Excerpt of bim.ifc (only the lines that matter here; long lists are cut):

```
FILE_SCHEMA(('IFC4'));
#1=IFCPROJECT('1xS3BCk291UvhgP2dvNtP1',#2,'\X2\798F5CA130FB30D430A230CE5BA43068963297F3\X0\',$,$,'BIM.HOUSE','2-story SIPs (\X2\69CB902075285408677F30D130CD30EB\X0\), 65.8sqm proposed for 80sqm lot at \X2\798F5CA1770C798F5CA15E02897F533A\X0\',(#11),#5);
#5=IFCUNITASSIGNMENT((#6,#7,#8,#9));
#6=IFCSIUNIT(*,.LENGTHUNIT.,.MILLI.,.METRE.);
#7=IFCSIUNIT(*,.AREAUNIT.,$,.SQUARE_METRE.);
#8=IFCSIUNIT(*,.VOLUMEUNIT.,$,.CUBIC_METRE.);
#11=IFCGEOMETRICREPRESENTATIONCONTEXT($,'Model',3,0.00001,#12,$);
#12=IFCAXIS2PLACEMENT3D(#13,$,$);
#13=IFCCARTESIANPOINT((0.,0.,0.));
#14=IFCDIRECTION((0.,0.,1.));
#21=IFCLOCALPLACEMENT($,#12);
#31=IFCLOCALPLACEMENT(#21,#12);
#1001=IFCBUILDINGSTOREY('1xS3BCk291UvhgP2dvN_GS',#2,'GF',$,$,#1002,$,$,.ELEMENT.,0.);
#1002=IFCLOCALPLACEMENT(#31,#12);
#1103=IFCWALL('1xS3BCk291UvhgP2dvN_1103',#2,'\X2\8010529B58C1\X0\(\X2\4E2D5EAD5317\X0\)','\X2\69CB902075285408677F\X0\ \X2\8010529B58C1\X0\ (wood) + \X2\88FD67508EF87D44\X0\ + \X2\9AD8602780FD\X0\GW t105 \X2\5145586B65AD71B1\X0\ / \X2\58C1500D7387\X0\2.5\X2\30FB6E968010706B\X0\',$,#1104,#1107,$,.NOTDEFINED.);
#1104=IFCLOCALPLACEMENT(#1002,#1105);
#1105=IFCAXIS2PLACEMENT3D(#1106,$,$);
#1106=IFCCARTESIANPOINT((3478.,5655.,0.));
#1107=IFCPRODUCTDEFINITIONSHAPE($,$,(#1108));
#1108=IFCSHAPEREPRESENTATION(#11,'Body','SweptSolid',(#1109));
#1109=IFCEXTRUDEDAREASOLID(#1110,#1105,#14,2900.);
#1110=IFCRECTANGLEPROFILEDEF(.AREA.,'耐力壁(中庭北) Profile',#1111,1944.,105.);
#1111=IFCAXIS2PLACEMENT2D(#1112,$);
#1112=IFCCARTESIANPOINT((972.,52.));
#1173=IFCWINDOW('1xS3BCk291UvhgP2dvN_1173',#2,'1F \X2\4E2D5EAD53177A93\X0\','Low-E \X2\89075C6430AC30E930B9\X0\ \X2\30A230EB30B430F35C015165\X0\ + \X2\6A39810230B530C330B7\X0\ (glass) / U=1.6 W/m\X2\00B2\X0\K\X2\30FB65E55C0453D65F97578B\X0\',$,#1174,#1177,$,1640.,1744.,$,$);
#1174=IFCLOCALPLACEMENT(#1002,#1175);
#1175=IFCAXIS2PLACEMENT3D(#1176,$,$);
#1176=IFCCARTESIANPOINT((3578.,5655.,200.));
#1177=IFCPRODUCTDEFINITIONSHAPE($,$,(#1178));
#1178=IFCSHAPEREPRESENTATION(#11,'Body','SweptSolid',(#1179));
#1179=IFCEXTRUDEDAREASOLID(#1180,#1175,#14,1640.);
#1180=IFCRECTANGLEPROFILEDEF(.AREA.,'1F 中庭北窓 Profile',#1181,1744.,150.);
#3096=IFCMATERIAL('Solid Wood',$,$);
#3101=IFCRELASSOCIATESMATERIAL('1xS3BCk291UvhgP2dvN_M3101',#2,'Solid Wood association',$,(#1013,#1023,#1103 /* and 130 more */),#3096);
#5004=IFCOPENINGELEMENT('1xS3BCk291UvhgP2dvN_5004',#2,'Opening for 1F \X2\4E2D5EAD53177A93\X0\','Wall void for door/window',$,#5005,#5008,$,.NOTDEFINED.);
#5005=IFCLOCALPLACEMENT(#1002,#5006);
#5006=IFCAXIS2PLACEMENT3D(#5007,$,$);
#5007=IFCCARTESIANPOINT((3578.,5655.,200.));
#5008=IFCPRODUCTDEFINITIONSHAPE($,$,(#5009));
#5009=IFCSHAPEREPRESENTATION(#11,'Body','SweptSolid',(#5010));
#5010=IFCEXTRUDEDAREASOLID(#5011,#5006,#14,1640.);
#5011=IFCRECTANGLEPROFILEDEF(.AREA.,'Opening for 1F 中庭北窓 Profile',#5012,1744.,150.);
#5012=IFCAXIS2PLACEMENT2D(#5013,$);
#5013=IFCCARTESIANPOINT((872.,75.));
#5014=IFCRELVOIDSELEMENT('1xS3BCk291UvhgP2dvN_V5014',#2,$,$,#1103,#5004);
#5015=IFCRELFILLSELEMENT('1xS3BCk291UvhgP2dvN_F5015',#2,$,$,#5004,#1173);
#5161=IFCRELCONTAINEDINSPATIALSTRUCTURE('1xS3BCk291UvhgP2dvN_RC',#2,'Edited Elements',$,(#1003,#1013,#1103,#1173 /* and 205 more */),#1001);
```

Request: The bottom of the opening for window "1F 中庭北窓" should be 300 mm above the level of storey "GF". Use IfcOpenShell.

```python
import numpy as np
import ifcopenshell
import ifcopenshell.api.geometry
import ifcopenshell.geom
import ifcopenshell.util.element
import ifcopenshell.util.placement
import ifcopenshell.util.shape
import ifcopenshell.util.unit

model = ifcopenshell.open("bim.ifc")
unit_scale = ifcopenshell.util.unit.calculate_unit_scale(model)

window = model.by_guid("1xS3BCk291UvhgP2dvN_1173")
opening = window.FillsVoids[0].RelatingOpeningElement
storey = ifcopenshell.util.element.get_container(window, ifc_class="IfcBuildingStorey")
level = ifcopenshell.util.placement.get_local_placement(storey.ObjectPlacement)[2, 3]

# The opening's origin need not be at the sill, so measure its lowest point.
shape = ifcopenshell.geom.create_shape(ifcopenshell.geom.settings(), opening)
bottom = ifcopenshell.util.shape.get_shape_bottom_elevation(shape, shape.geometry) / unit_scale
dz = level + 0.3 / unit_scale - bottom

shift = np.array([0.0, 0.0, dz])
# The window is not placed relative to its opening, so move both.
for product in (opening, window):
    matrix = ifcopenshell.util.placement.get_local_placement(product.ObjectPlacement)
    matrix[:3, 3] += shift
    ifcopenshell.api.geometry.edit_object_placement(model, product=product, matrix=matrix, is_si=False)

print(f"moved by {dz * unit_scale:+.3f} m")

model.write("bim_edited.ifc")
```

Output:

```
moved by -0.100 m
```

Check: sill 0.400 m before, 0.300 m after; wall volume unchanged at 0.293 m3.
